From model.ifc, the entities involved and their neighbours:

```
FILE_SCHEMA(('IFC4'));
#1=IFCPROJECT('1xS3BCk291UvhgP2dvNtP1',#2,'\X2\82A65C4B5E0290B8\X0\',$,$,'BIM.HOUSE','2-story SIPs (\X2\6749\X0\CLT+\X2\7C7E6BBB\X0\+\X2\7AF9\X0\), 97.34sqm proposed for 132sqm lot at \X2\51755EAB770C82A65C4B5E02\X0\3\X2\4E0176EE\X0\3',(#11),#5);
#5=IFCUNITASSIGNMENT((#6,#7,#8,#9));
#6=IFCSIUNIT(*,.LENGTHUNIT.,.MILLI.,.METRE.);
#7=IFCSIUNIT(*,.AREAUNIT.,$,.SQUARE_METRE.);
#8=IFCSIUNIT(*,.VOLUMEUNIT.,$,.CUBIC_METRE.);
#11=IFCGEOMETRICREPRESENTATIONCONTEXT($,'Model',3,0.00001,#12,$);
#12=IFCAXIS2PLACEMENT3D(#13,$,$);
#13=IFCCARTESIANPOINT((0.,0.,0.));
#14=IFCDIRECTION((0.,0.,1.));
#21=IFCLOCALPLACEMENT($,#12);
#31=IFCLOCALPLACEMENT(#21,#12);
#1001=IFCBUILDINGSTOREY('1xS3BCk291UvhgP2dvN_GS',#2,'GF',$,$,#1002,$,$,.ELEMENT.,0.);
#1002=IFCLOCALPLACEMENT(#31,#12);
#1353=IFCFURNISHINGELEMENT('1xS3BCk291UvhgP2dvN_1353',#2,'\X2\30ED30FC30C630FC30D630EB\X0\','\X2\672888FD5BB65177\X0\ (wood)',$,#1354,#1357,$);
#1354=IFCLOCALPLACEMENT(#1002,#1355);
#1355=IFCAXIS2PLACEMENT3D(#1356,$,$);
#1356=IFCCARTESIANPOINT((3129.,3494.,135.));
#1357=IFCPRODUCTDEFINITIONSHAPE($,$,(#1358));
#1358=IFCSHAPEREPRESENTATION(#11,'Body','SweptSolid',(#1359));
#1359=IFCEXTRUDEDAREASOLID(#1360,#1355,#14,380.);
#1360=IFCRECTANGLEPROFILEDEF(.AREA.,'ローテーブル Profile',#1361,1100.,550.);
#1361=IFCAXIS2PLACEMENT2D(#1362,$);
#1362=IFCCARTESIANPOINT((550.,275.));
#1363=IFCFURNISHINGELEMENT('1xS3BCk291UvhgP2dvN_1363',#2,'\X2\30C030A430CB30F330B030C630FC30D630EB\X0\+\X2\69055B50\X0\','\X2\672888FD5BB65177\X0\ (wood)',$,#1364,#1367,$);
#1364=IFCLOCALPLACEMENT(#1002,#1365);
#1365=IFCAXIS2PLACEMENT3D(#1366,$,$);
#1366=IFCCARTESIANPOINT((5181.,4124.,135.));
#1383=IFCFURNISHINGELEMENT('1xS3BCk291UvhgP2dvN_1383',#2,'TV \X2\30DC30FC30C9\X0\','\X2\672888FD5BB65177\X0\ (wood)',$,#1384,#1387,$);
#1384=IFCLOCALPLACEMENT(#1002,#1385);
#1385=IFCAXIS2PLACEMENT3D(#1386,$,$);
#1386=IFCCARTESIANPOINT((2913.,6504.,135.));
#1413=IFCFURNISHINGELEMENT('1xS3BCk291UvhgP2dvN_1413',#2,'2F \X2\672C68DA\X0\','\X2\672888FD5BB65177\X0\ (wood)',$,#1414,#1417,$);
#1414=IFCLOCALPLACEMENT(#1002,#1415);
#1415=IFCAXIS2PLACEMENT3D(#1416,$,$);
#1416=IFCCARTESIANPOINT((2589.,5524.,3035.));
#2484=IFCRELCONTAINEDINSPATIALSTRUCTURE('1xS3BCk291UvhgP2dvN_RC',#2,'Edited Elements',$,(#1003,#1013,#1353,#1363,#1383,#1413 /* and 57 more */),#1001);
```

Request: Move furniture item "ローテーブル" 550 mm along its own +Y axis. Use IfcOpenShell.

```python
import ifcopenshell
import ifcopenshell.api.geometry
import ifcopenshell.util.placement
import ifcopenshell.util.unit

model = ifcopenshell.open("model.ifc")
unit_scale = ifcopenshell.util.unit.calculate_unit_scale(model)

item = model.by_guid("1xS3BCk291UvhgP2dvN_1353")
matrix = ifcopenshell.util.placement.get_local_placement(item.ObjectPlacement)
matrix[:3, 3] += matrix[:3, 1] * 0.55 / unit_scale
ifcopenshell.api.geometry.edit_object_placement(model, product=item, matrix=matrix, is_si=False)

print(ifcopenshell.util.placement.get_local_placement(item.ObjectPlacement).round(3) + 0.0)

model.write("model_rev.ifc")
```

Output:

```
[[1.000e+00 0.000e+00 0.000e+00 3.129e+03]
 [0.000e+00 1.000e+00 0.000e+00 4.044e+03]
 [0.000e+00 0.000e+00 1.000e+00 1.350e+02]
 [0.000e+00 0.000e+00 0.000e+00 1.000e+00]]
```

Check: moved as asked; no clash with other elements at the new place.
